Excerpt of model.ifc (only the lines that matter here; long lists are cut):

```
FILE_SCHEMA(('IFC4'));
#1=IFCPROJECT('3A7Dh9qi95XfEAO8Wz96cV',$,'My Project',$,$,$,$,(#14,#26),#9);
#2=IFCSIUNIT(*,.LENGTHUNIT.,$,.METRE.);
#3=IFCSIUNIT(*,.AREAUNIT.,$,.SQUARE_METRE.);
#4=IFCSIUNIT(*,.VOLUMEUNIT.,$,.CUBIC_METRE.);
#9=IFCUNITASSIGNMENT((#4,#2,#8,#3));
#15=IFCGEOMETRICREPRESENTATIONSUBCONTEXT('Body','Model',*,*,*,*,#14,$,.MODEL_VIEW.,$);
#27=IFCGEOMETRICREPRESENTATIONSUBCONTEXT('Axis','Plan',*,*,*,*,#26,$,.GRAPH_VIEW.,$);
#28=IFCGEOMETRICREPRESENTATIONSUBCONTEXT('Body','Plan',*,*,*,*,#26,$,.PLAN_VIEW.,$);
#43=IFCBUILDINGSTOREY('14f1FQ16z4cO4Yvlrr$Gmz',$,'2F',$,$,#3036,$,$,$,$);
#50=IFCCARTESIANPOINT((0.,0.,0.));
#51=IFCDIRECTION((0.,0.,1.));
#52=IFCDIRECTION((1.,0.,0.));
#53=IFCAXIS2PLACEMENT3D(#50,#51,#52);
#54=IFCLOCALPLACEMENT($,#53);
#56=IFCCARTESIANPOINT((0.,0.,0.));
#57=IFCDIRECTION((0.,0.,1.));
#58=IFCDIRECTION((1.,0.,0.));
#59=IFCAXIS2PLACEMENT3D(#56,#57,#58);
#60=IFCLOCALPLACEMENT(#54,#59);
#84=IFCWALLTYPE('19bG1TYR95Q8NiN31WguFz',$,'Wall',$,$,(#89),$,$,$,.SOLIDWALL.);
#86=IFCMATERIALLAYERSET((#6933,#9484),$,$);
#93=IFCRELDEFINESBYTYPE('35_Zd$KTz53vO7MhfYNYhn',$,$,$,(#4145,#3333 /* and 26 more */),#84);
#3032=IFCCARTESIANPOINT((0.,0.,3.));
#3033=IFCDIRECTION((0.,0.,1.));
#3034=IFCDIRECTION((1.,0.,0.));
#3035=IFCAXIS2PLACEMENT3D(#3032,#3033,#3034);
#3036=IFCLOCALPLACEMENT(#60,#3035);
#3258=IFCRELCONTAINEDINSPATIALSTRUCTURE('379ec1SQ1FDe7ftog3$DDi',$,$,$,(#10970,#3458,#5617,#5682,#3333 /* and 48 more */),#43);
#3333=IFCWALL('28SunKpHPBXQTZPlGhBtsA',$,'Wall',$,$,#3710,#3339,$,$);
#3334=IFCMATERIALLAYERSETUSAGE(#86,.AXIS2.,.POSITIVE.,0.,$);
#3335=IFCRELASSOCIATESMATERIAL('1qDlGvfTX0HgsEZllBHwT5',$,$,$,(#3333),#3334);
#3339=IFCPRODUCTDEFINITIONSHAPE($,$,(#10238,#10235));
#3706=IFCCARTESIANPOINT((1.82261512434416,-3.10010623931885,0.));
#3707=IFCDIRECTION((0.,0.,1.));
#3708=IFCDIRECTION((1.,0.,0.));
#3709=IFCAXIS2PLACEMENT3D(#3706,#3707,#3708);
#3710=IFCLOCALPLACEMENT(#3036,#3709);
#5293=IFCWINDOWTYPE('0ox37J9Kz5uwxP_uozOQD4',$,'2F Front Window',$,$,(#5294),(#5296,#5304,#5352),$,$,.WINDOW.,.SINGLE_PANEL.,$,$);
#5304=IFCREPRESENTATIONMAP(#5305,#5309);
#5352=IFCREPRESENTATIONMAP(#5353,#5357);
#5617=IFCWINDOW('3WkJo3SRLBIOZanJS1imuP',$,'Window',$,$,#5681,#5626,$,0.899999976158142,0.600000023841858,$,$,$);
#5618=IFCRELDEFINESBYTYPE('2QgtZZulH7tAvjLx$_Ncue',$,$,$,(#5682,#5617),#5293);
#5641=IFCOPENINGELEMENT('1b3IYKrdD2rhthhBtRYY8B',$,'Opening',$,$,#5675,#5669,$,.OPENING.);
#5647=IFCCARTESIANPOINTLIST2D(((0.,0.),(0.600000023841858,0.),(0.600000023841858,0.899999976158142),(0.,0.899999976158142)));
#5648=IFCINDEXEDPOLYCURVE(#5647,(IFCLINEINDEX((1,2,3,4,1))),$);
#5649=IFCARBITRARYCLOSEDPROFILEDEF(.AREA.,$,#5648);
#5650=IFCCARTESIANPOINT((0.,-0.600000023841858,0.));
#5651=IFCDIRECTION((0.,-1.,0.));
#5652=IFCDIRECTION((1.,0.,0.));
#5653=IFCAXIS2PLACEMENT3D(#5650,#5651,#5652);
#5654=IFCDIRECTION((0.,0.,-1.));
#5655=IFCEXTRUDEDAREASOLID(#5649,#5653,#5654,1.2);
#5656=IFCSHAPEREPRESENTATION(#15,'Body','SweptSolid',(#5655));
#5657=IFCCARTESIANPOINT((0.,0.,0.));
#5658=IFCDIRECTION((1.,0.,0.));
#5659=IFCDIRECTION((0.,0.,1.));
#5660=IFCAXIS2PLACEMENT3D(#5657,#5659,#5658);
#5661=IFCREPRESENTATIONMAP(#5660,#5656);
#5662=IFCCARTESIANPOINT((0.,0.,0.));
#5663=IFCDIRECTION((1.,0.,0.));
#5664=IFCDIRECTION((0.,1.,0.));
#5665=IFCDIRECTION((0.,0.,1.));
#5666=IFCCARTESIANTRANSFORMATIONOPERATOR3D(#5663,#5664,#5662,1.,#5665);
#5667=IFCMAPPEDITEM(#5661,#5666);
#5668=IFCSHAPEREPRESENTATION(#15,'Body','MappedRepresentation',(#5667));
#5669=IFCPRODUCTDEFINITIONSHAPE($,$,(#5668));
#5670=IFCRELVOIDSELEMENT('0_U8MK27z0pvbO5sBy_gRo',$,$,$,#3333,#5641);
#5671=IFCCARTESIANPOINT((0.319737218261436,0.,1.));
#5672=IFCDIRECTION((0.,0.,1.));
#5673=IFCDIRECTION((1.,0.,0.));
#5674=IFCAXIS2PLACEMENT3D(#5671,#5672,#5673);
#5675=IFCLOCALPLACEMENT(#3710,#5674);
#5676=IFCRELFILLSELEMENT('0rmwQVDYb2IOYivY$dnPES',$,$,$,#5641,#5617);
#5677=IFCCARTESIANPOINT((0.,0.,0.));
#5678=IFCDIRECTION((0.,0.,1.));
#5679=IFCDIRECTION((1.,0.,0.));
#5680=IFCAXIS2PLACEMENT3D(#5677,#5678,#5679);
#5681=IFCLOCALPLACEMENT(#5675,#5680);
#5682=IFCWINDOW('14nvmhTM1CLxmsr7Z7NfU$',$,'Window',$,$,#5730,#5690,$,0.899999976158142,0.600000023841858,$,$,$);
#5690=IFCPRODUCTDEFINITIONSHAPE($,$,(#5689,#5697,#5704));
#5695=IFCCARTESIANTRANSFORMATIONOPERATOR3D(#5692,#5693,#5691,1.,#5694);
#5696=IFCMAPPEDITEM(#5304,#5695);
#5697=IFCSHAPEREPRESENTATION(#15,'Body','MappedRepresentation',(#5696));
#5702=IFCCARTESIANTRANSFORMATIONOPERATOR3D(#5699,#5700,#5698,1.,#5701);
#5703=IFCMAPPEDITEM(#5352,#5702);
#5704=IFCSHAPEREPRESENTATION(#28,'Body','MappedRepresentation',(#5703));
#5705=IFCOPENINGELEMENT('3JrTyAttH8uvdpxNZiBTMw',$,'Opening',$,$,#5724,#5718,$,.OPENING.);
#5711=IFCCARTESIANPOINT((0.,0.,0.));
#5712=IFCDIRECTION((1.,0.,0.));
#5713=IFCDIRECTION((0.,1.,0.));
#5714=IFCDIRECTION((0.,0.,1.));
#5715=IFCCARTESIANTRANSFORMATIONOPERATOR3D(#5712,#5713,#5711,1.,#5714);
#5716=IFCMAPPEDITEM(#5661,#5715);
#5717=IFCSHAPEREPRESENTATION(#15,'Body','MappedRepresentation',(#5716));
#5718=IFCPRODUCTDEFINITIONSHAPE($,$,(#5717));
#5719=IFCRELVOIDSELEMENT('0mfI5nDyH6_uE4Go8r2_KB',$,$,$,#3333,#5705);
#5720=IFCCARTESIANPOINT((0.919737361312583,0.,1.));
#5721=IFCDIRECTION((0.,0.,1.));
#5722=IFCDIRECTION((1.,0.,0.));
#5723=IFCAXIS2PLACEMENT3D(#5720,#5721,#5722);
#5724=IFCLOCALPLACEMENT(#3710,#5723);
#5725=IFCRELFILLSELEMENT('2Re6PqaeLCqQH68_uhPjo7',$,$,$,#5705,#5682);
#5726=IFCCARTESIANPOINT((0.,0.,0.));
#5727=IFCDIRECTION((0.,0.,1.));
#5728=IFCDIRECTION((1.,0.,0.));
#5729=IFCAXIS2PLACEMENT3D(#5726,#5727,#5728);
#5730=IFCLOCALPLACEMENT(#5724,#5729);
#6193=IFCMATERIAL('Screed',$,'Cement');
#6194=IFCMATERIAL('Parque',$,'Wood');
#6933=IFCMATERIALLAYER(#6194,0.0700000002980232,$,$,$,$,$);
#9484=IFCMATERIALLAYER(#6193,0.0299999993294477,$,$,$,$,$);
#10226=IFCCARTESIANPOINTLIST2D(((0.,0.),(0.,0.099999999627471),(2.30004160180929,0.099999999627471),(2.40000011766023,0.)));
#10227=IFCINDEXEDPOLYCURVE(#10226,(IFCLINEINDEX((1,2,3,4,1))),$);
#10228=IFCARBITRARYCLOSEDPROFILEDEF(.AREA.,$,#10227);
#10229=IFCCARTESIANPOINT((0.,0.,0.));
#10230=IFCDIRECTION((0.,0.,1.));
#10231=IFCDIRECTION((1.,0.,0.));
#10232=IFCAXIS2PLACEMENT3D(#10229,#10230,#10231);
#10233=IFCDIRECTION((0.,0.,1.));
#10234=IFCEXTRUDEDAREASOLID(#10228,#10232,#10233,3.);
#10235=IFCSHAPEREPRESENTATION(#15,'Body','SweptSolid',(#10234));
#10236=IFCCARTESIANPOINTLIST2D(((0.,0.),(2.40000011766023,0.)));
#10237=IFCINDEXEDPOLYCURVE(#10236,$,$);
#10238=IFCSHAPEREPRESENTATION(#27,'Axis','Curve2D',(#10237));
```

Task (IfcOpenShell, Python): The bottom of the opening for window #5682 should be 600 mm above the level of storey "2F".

```python
import numpy as np
import ifcopenshell
import ifcopenshell.api.geometry
import ifcopenshell.geom
import ifcopenshell.util.element
import ifcopenshell.util.placement
import ifcopenshell.util.shape
import ifcopenshell.util.unit

model = ifcopenshell.open("model.ifc")
unit_scale = ifcopenshell.util.unit.calculate_unit_scale(model)

window = model.by_id(5682)
opening = window.FillsVoids[0].RelatingOpeningElement
storey = ifcopenshell.util.element.get_container(window, ifc_class="IfcBuildingStorey")
level = ifcopenshell.util.placement.get_local_placement(storey.ObjectPlacement)[2, 3]

# The opening's origin need not be at the sill, so measure its lowest point.
shape = ifcopenshell.geom.create_shape(ifcopenshell.geom.settings(), opening)
bottom = ifcopenshell.util.shape.get_shape_bottom_elevation(shape, shape.geometry) / unit_scale
dz = level + 0.6 - bottom

shift = np.array([0.0, 0.0, dz])
# The window is placed relative to its opening, so it follows when the opening moves.
matrix = ifcopenshell.util.placement.get_local_placement(opening.ObjectPlacement)
matrix[:3, 3] += shift
ifcopenshell.api.geometry.edit_object_placement(
    model, product=opening, matrix=matrix, is_si=False, should_transform_children=True
)

print(f"moved by {dz * unit_scale:+.3f} m")

model.write("model-out.ifc")
```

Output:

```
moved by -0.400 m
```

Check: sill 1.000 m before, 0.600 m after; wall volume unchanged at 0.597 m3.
